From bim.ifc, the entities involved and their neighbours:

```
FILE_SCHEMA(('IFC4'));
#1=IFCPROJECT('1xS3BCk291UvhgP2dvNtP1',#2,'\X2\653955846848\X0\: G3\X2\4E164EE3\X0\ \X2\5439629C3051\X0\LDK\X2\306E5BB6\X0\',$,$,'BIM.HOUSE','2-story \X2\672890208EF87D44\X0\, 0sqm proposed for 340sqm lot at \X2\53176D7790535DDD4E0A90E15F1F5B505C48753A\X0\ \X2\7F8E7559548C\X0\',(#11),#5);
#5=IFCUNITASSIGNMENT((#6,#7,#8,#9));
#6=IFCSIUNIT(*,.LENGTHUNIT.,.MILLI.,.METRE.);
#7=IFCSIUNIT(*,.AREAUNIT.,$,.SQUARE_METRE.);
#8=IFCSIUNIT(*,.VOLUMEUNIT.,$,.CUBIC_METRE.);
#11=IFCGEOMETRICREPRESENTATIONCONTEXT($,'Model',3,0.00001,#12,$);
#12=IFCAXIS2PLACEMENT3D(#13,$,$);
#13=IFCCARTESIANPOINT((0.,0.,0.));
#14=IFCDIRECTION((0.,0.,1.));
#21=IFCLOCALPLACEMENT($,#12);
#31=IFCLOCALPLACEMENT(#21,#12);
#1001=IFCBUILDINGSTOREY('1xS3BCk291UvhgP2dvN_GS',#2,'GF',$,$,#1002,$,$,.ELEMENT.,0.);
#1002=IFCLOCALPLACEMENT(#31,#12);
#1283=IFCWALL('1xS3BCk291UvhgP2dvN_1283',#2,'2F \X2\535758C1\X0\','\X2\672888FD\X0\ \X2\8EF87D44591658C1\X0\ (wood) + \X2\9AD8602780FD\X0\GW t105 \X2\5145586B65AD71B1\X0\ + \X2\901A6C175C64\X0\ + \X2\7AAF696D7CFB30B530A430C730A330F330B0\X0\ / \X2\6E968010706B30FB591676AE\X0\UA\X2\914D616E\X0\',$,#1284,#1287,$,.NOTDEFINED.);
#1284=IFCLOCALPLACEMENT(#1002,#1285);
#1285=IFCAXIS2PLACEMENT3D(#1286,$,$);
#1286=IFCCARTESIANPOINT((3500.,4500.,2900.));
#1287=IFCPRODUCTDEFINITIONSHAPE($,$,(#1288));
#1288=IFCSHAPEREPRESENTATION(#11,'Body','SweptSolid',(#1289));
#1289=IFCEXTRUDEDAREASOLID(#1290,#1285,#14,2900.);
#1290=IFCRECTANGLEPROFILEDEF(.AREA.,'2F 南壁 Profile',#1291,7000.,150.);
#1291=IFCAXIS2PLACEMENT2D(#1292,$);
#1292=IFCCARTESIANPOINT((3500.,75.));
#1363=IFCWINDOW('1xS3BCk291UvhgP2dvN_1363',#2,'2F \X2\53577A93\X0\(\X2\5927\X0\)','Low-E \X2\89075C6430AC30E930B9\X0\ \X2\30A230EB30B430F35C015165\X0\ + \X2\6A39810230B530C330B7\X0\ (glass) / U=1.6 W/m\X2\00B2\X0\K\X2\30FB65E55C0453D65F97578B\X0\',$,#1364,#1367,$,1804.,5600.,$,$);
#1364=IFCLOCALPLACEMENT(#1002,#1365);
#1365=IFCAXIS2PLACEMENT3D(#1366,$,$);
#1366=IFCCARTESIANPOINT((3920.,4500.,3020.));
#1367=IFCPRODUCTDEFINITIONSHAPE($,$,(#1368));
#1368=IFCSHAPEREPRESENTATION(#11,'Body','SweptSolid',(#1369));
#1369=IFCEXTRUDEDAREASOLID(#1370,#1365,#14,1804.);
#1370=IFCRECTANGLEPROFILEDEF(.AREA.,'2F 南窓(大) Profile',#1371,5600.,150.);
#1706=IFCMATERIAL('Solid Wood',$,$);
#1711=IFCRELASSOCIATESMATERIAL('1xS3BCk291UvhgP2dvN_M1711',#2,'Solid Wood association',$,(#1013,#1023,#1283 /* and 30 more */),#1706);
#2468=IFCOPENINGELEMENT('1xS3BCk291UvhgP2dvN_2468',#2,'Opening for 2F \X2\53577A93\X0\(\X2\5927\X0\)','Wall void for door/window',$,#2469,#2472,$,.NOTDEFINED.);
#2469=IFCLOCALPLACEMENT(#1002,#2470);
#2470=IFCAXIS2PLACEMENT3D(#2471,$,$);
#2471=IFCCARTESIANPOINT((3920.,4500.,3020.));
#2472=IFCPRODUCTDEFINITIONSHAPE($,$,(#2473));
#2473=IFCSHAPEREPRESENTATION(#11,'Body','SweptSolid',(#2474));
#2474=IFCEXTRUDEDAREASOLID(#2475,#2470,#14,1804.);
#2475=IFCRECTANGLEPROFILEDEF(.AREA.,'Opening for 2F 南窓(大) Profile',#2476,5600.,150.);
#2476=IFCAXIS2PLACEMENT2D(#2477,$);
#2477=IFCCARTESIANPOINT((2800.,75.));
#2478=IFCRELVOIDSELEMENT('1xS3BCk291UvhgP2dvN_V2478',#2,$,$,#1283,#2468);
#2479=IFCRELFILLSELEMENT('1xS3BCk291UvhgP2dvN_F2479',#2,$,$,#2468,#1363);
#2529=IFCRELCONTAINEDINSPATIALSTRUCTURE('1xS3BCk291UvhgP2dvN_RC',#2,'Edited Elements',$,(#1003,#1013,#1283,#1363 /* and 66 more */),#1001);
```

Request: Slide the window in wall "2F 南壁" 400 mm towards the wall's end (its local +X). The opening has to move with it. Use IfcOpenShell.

```python
import ifcopenshell
import ifcopenshell.api.geometry
import ifcopenshell.util.placement

model = ifcopenshell.open("bim.ifc")

window = model.by_guid("1xS3BCk291UvhgP2dvN_1363")
opening = window.FillsVoids[0].RelatingOpeningElement
wall = opening.VoidsElements[0].RelatingBuildingElement

wall_matrix = ifcopenshell.util.placement.get_local_placement(wall.ObjectPlacement)
shift = wall_matrix[:3, 0] * 400.0
before = ifcopenshell.util.placement.get_local_placement(window.ObjectPlacement)[:3, 3].copy()

# The window is not placed relative to its opening, so move both.
for product in (opening, window):
    matrix = ifcopenshell.util.placement.get_local_placement(product.ObjectPlacement)
    matrix[:3, 3] += shift
    ifcopenshell.api.geometry.edit_object_placement(model, product=product, matrix=matrix, is_si=False)

after = ifcopenshell.util.placement.get_local_placement(window.ObjectPlacement)[:3, 3]
print("window moved by", (after - before).round(3) + 0.0)

model.write("bim-out.ifc")
```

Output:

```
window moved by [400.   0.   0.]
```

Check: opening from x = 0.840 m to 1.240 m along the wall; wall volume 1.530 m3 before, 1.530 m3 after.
